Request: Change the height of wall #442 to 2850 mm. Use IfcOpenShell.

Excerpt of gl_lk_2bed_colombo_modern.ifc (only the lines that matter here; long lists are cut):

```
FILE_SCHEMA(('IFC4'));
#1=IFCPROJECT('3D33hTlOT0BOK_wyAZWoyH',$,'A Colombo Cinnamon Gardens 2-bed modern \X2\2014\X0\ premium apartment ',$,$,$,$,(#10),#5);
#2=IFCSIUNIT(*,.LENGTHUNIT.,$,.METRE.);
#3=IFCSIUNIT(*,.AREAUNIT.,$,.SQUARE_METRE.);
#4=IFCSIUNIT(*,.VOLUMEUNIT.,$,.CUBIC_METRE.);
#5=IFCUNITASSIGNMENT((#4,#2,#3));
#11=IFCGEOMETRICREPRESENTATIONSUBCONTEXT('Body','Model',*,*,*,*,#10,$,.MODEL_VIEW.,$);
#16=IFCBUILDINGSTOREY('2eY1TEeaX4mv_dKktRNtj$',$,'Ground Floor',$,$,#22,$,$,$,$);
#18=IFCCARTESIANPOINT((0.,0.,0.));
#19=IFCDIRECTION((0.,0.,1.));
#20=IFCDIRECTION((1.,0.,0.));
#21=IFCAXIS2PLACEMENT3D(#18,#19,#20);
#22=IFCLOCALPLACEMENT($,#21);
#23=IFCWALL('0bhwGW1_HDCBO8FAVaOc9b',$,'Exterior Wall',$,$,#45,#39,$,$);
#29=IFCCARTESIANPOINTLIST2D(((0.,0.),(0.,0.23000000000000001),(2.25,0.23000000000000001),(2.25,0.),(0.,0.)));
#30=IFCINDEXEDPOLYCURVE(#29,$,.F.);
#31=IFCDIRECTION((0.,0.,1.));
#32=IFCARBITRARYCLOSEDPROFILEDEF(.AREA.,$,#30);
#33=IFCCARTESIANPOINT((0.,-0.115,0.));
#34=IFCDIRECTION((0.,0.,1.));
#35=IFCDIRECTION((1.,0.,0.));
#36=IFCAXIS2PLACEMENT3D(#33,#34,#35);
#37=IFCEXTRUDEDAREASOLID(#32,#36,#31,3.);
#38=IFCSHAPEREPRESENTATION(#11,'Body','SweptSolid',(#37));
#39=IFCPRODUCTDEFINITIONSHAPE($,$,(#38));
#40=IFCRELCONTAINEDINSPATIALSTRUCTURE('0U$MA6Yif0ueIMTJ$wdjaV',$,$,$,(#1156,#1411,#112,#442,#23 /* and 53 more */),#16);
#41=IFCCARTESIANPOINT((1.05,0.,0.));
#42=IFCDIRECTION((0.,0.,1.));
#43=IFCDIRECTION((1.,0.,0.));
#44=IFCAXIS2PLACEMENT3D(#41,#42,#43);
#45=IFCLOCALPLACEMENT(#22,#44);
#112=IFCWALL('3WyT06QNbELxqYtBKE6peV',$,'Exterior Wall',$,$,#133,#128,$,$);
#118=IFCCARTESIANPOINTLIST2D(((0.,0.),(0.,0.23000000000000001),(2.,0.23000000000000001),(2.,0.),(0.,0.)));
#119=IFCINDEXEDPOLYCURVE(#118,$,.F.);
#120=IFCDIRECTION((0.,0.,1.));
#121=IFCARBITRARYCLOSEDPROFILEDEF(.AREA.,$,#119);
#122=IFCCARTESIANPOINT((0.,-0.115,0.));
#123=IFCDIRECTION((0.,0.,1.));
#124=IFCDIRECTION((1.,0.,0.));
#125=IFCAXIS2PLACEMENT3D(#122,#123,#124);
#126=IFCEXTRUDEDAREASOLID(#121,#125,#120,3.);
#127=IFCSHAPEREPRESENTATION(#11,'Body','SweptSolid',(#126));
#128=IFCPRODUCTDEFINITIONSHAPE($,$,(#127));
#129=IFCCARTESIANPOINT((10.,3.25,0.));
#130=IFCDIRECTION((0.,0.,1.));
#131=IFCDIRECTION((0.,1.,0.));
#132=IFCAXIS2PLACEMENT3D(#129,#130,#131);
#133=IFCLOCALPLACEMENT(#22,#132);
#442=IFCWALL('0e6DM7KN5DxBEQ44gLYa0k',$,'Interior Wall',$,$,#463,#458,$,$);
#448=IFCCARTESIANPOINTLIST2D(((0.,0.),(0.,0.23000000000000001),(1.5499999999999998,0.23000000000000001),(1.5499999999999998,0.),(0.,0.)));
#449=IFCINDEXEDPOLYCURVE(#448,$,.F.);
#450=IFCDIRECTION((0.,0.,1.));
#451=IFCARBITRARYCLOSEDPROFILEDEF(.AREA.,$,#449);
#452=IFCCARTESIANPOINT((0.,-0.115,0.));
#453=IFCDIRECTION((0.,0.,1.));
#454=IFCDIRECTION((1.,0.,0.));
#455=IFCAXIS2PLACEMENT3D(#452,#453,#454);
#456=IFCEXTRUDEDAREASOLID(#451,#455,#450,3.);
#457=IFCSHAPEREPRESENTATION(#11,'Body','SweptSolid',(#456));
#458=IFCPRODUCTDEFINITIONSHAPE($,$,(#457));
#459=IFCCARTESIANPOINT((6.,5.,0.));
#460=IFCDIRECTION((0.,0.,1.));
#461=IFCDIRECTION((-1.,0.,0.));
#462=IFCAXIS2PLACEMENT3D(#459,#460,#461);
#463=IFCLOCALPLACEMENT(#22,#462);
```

```python
import ifcopenshell
import ifcopenshell.geom
import ifcopenshell.util.representation
import ifcopenshell.util.shape
import ifcopenshell.util.unit

model = ifcopenshell.open("gl_lk_2bed_colombo_modern.ifc")
unit_scale = ifcopenshell.util.unit.calculate_unit_scale(model)
settings = ifcopenshell.geom.settings()


def volume(element):
    """Net volume in cubic metres, openings subtracted."""
    shape = ifcopenshell.geom.create_shape(settings, element)
    return ifcopenshell.util.shape.get_volume(shape.geometry)


wall = model.by_id(442)
before = volume(wall)

body = ifcopenshell.util.representation.get_representation(wall, "Model", "Body")
solid = body.Items[0]
old_height = solid.Depth
solid.Depth = 2.85 / unit_scale
after = volume(wall)

print(f"height {old_height:g} -> {solid.Depth:g}, volume {before:.3f} -> {after:.3f} m3")

model.write("gl_lk_2bed_colombo_modern_edited.ifc")
```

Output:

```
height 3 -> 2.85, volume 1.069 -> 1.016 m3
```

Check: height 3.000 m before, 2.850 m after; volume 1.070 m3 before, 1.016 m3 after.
